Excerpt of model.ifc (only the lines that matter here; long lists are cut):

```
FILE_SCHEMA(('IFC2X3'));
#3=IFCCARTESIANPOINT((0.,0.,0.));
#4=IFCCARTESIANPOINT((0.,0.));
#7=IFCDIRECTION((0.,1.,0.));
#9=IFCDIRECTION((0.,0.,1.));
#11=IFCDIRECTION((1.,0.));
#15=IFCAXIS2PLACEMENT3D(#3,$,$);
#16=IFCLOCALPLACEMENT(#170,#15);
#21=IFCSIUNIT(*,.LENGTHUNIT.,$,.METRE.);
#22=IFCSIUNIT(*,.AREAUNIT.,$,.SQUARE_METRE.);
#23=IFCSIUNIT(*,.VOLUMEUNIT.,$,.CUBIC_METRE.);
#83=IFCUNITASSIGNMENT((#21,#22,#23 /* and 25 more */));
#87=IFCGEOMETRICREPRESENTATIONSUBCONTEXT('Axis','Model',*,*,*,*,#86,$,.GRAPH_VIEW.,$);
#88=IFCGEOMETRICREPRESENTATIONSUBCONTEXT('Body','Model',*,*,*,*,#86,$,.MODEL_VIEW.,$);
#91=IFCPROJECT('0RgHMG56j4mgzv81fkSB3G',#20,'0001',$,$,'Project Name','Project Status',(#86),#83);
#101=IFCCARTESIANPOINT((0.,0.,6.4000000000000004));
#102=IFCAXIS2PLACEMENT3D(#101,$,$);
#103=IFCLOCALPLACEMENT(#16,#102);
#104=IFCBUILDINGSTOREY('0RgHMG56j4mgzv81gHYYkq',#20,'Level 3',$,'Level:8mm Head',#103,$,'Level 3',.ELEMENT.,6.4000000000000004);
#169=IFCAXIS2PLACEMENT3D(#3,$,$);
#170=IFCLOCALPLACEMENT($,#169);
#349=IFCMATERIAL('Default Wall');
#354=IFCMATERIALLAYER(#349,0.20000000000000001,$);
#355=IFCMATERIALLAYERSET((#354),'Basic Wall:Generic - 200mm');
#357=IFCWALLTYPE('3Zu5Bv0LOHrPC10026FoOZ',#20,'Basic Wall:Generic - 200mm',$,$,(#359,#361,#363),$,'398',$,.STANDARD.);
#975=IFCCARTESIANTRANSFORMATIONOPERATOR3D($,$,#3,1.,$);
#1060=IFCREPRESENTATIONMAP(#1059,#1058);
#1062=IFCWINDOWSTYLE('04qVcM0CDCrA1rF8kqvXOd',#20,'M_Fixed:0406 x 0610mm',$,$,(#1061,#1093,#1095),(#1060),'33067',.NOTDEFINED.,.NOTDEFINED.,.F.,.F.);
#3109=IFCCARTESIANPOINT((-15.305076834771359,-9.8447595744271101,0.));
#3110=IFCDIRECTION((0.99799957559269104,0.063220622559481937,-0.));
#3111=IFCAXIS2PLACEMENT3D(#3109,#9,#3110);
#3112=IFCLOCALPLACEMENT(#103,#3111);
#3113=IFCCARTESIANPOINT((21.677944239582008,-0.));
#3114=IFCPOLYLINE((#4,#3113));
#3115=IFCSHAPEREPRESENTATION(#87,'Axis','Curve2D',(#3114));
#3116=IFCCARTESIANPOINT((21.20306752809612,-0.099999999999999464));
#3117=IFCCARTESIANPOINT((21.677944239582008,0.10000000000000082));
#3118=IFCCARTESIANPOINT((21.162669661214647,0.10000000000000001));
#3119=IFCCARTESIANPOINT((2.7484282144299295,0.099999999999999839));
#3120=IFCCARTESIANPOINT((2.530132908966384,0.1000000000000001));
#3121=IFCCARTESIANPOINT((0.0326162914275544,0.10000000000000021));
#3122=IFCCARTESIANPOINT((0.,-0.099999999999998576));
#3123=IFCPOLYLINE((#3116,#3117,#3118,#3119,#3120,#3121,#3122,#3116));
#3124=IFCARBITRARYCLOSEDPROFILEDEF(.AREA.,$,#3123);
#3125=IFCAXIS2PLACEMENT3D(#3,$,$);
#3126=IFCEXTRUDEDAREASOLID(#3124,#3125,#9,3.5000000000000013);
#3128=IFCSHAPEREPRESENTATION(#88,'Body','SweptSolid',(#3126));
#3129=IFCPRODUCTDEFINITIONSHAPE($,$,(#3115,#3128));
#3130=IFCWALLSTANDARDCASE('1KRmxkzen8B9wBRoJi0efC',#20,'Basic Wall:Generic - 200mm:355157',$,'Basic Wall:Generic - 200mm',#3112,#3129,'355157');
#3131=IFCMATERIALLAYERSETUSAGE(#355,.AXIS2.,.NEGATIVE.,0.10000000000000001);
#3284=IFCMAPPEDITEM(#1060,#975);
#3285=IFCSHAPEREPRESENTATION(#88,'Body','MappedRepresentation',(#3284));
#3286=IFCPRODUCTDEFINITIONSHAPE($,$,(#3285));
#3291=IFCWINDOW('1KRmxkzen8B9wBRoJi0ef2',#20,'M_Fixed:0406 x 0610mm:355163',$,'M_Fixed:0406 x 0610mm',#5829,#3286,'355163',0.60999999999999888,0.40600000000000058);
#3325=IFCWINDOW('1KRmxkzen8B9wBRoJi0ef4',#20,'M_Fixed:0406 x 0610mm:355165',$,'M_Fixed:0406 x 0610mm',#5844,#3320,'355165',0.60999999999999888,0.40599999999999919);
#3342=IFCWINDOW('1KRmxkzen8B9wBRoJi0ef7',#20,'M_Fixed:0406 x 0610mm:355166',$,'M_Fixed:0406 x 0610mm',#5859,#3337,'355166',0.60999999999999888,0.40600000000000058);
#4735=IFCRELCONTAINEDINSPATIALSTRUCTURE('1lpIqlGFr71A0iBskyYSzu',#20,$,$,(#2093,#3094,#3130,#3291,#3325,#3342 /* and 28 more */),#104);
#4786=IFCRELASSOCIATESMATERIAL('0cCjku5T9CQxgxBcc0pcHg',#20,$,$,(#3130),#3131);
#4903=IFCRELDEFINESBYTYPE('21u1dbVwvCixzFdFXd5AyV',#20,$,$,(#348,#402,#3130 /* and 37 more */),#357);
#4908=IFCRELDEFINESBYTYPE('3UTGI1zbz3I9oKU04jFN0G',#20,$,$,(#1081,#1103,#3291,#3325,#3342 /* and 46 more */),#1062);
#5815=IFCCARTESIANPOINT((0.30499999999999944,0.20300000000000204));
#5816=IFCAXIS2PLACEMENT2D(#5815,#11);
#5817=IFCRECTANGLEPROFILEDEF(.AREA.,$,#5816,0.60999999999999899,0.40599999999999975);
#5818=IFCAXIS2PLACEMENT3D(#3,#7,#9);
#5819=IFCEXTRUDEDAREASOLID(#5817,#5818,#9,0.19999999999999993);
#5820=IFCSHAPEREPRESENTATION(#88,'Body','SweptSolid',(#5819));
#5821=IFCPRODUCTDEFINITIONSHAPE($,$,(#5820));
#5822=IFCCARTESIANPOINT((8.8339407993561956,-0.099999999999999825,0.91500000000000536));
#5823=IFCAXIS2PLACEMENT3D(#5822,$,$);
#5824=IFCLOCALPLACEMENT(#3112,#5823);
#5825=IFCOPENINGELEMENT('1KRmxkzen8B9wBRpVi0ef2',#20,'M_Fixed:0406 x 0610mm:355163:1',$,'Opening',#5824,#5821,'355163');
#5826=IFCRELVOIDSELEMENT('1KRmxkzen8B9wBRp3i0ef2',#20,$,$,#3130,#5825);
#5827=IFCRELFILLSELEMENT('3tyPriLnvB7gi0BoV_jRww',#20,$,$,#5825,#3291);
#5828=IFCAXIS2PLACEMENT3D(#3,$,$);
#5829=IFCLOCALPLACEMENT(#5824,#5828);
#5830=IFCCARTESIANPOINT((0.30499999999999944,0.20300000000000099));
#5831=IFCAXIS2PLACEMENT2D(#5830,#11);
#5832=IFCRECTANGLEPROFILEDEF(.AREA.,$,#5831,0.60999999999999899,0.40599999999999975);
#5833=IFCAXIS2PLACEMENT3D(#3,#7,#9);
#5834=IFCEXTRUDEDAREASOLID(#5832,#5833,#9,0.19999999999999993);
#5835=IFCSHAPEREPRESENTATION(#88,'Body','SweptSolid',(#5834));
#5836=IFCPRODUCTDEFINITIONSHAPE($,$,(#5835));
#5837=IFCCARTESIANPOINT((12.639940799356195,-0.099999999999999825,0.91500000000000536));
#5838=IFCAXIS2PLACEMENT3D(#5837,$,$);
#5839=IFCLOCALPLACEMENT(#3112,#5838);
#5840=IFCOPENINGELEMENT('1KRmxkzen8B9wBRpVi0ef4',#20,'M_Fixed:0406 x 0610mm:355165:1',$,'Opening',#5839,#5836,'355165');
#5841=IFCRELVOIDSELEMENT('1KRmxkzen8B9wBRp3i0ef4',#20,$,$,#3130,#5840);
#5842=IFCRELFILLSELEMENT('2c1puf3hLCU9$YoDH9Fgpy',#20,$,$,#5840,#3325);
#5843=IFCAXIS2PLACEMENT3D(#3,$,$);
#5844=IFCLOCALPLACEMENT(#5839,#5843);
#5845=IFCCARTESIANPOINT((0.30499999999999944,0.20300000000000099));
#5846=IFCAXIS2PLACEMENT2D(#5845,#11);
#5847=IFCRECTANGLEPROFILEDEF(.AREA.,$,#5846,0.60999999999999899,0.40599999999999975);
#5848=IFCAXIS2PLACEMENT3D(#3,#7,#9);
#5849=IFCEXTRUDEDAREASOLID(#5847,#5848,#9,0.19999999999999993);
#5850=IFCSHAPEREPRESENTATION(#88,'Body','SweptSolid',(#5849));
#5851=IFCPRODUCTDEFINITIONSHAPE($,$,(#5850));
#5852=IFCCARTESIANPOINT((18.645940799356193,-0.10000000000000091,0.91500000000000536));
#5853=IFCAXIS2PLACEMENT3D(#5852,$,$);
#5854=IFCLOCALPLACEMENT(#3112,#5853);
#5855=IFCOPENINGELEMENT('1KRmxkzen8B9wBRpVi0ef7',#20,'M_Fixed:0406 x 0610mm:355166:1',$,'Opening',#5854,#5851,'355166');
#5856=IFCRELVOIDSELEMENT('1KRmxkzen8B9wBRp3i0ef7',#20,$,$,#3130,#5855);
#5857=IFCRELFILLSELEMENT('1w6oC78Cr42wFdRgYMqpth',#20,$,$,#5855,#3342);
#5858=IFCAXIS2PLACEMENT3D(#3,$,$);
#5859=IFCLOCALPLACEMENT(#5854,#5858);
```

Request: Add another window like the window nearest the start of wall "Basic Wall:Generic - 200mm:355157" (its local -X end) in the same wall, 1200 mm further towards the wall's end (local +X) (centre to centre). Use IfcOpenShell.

```python
import ifcopenshell
import ifcopenshell.api.feature
import ifcopenshell.api.geometry
import ifcopenshell.api.root
import ifcopenshell.geom
import ifcopenshell.util.element
import ifcopenshell.util.placement
import ifcopenshell.util.shape

model = ifcopenshell.open("model.ifc")
settings = ifcopenshell.geom.settings()


def volume(element):
    """Net volume in cubic metres, openings subtracted."""
    shape = ifcopenshell.geom.create_shape(settings, element)
    return ifcopenshell.util.shape.get_volume(shape.geometry)


def reuse_history(source, copy):
    """copy_class also copies each property set's owner history, people and application; keep the originals."""
    for rel in copy.IsDefinedBy:
        if rel.is_a("IfcRelDefinesByProperties") and (history := rel.RelatingPropertyDefinition.OwnerHistory):
            rel.RelatingPropertyDefinition.OwnerHistory = source.OwnerHistory
            ifcopenshell.util.element.remove_deep2(model, history)


window = model.by_id(3291)
opening = window.FillsVoids[0].RelatingOpeningElement
wall = opening.VoidsElements[0].RelatingBuildingElement
before = volume(wall)
shift = ifcopenshell.util.placement.get_local_placement(wall.ObjectPlacement)[:3, 0] * 1.2

# copy_class copies the void relationship, type, container and properties, but no geometry.
new_opening = ifcopenshell.api.root.copy_class(model, product=opening)
new_opening.Representation = ifcopenshell.util.element.copy_deep(
    model, opening.Representation, exclude=["IfcGeometricRepresentationContext", "IfcRepresentationMap"]
)
new_opening.Name = "M_Fixed:0406 x 0610mm"
new_opening.Tag = None
new_window = ifcopenshell.api.root.copy_class(model, product=window)
new_window.Representation = ifcopenshell.util.element.copy_deep(
    model, window.Representation, exclude=["IfcGeometricRepresentationContext", "IfcRepresentationMap"]
)
new_window.Name = "M_Fixed:0406 x 0610mm"
new_window.Tag = None
reuse_history(window, new_window)
fills = ifcopenshell.api.feature.add_filling(model, opening=new_opening, element=new_window)
fills.OwnerHistory = new_window.OwnerHistory  # required in IFC2X3

for old, new in ((opening, new_opening), (window, new_window)):
    matrix = ifcopenshell.util.placement.get_local_placement(old.ObjectPlacement)
    matrix[:3, 3] += shift
    ifcopenshell.api.geometry.edit_object_placement(model, product=new, matrix=matrix, is_si=False)

after = volume(wall)

print(f"wall volume {before:.3f} -> {after:.3f} m3")

model.write("model_edited.ifc")
```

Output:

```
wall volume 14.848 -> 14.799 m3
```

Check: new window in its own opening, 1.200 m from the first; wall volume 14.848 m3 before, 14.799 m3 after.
